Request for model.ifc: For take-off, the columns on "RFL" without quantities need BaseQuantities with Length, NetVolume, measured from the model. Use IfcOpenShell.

First a look at what the model holds.

```python
import ifcopenshell
import ifcopenshell.util.element
import ifcopenshell.util.unit

model = ifcopenshell.open("model.ifc")
print(model.schema)
for unit_type in ("LENGTHUNIT", "AREAUNIT", "VOLUMEUNIT"):
    print(unit_type, ifcopenshell.util.unit.calculate_unit_scale(model, unit_type))
storey = next(s for s in model.by_type("IfcBuildingStorey") if s.Name == "RFL")
columns = [e for e in ifcopenshell.util.element.get_decomposition(storey) if e.is_a("IfcColumn")]
for e in sorted(columns, key=lambda e: e.id()):
    print(e.id(), e.is_a(), e.Name, list(ifcopenshell.util.element.get_psets(e, qtos_only=True)), sep=" | ")
```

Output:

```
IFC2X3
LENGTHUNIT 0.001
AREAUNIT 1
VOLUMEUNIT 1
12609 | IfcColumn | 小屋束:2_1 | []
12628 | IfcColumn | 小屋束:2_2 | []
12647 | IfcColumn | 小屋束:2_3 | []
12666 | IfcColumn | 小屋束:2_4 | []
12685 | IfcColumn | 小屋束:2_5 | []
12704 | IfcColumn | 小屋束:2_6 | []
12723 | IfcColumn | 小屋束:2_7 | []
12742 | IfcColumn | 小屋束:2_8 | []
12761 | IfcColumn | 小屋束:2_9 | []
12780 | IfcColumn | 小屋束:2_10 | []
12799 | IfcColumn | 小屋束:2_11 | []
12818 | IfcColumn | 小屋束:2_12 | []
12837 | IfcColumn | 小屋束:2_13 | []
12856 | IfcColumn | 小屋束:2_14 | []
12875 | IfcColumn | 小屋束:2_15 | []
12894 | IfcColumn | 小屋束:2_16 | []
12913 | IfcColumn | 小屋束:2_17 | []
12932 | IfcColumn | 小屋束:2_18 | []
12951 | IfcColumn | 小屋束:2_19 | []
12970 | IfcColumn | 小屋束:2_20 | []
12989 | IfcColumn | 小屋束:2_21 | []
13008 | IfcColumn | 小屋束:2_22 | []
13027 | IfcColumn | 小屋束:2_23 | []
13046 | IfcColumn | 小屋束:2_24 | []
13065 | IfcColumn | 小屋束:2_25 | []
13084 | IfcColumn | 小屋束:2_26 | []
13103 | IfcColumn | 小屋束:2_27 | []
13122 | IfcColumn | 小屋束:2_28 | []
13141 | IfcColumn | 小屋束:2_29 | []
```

```python
import ifcopenshell
import ifcopenshell.api.pset
import ifcopenshell.geom
import ifcopenshell.util.element
import ifcopenshell.util.shape
import ifcopenshell.util.unit

model = ifcopenshell.open("model.ifc")
unit_scale = ifcopenshell.util.unit.calculate_unit_scale(model)
volume_scale = ifcopenshell.util.unit.calculate_unit_scale(model, "VOLUMEUNIT")
settings = ifcopenshell.geom.settings()

storey = next(s for s in model.by_type("IfcBuildingStorey") if s.Name == "RFL")
columns = [e for e in ifcopenshell.util.element.get_decomposition(storey) if e.is_a("IfcColumn")]

for e in sorted(columns, key=lambda e: e.id()):
    if ifcopenshell.util.element.get_psets(e, qtos_only=True, should_inherit=False):
        continue
    # Geometry comes back in metres, in the element's own axes.
    shape = ifcopenshell.geom.create_shape(settings, e)
    values = {
        "Length": ifcopenshell.util.shape.get_z(shape.geometry) / unit_scale,
        "NetVolume": ifcopenshell.util.shape.get_volume(shape.geometry) / volume_scale,
    }
    qto = ifcopenshell.api.pset.add_qto(model, product=e, name="BaseQuantities")
    ifcopenshell.api.pset.edit_qto(model, qto=qto, properties=values)
    print(e.id(), {k: round(v, 3) for k, v in values.items()})

model.write("model-out.ifc")
```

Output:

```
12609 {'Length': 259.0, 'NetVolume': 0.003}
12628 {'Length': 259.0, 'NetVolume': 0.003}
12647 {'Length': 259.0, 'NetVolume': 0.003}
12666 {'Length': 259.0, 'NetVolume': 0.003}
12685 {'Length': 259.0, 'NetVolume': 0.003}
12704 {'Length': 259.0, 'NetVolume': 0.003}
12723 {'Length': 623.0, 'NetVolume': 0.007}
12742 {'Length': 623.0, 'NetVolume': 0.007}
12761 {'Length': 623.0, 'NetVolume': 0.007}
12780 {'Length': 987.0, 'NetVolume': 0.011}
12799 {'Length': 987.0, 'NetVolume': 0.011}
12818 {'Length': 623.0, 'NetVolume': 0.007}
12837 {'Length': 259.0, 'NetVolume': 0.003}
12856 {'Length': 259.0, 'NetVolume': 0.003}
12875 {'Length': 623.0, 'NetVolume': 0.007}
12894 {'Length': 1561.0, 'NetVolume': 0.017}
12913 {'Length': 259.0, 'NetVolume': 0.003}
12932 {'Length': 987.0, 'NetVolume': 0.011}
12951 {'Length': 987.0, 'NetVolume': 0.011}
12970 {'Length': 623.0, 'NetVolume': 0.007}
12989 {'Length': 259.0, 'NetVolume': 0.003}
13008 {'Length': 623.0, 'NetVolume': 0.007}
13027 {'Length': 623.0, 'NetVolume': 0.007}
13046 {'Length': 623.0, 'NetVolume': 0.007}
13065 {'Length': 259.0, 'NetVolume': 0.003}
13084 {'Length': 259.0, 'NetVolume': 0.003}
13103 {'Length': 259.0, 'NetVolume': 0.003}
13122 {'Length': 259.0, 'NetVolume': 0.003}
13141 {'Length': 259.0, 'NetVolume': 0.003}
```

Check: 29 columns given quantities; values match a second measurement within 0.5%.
